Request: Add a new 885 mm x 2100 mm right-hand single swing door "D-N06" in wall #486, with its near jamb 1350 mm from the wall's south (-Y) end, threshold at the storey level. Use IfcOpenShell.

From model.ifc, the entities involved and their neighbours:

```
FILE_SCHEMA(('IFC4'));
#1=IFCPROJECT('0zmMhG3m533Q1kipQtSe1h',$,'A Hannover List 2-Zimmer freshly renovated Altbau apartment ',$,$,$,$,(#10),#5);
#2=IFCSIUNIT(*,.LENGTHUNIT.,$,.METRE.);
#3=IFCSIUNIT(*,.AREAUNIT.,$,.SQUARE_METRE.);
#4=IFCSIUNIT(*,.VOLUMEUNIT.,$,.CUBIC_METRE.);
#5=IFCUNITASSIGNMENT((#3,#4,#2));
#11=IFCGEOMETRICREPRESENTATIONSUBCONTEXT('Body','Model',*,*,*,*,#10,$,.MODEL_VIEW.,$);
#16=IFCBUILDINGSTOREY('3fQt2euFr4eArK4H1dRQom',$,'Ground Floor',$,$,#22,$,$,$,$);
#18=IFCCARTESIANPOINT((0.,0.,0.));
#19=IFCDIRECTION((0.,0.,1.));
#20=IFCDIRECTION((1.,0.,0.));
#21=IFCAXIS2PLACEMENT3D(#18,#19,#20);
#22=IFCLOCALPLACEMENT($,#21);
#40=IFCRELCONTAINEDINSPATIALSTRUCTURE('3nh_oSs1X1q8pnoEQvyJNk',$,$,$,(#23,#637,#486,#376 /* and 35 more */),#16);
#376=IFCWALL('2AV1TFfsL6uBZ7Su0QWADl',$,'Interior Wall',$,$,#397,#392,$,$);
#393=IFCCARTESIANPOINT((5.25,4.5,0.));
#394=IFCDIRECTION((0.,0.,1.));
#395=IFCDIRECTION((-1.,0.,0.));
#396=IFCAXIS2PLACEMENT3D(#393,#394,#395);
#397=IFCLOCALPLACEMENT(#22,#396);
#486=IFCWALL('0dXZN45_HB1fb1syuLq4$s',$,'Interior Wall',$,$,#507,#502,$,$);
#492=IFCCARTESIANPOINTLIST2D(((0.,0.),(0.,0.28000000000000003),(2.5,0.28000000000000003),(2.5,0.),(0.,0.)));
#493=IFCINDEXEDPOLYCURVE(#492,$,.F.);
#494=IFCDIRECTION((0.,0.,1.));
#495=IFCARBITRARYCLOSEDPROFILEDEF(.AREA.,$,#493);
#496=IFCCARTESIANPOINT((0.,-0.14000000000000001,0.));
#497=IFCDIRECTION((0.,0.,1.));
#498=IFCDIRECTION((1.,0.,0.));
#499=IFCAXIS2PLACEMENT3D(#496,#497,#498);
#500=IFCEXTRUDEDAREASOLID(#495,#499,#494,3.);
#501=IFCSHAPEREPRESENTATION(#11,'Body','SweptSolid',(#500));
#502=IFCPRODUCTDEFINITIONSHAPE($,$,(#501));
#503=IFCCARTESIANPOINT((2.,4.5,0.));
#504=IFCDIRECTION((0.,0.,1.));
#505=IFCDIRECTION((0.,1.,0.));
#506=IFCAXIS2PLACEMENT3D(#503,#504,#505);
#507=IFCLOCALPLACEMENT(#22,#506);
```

```python
import numpy as np
import ifcopenshell
import ifcopenshell.api.feature
import ifcopenshell.api.geometry
import ifcopenshell.api.root
import ifcopenshell.api.spatial
import ifcopenshell.geom
import ifcopenshell.util.element
import ifcopenshell.util.placement
import ifcopenshell.util.representation
import ifcopenshell.util.shape
import ifcopenshell.util.unit

model = ifcopenshell.open("model.ifc")
unit_scale = ifcopenshell.util.unit.calculate_unit_scale(model)
settings = ifcopenshell.geom.settings()


def volume(element):
    """Net volume in cubic metres, openings subtracted."""
    shape = ifcopenshell.geom.create_shape(settings, element)
    return ifcopenshell.util.shape.get_volume(shape.geometry)


wall = model.by_guid("0dXZN45_HB1fb1syuLq4$s")
storey = ifcopenshell.util.element.get_container(wall, ifc_class="IfcBuildingStorey")
context = ifcopenshell.util.representation.get_context(model, "Model", "Body", "MODEL_VIEW")
before = volume(wall)

width, height, from_end, sill = 0.885, 2.1, 1.35, 0.0  # metres

# The wall runs along its own X axis, and the end named is its -X end.
wall_shape = ifcopenshell.geom.create_shape(settings, wall)
x, y, z = ifcopenshell.util.shape.get_vertices(wall_shape.geometry).T
start = x.min() + from_end
face, thickness = float(y.min()), float(y.max() - y.min())
wall_matrix = ifcopenshell.util.placement.get_local_placement(wall.ObjectPlacement)
level = ifcopenshell.util.placement.get_local_placement(storey.ObjectPlacement)[2, 3]


def in_wall(x, y):
    """Placement at x, y metres in the wall's axes, at sill height."""
    matrix = wall_matrix.copy()
    matrix[:, 3] = wall_matrix @ np.array([x / unit_scale, y / unit_scale, 0.0, 1.0])
    matrix[2, 3] = level + sill / unit_scale
    return matrix


# Opening: a box that overshoots both wall faces by 50 mm.
opening = ifcopenshell.api.root.create_entity(model, ifc_class="IfcOpeningElement", predefined_type="OPENING")
box = ifcopenshell.api.geometry.add_wall_representation(
    model, context=context, length=width, height=height, thickness=thickness + 0.1
)
ifcopenshell.api.geometry.assign_representation(model, product=opening, representation=box)
ifcopenshell.api.geometry.edit_object_placement(model, product=opening, matrix=in_wall(start, face - 0.05), is_si=False)
ifcopenshell.api.feature.add_feature(model, feature=opening, element=wall)

door = ifcopenshell.api.root.create_entity(model, ifc_class="IfcDoor", name="D-N06", predefined_type="DOOR")
door.OverallWidth, door.OverallHeight = width / unit_scale, height / unit_scale
door.OperationType = "SINGLE_SWING_RIGHT"
body = ifcopenshell.api.geometry.add_door_representation(
    model,
    context=context,
    overall_width=door.OverallWidth,
    overall_height=door.OverallHeight,
    operation_type="SINGLE_SWING_RIGHT",
    lining_properties={"LiningDepth": thickness / unit_scale, "ThresholdDepth": thickness / unit_scale},
)
ifcopenshell.api.geometry.assign_representation(model, product=door, representation=body)
ifcopenshell.api.spatial.assign_container(model, products=[door], relating_structure=storey)
ifcopenshell.api.feature.add_filling(model, opening=opening, element=door)

# The lining spans the wall, so the door starts at the wall face.
ifcopenshell.api.geometry.edit_object_placement(model, product=door, matrix=in_wall(start, face), is_si=False)

after = volume(wall)

print(f"wall volume {before:.3f} -> {after:.3f} m3")

model.write("model_edited.ifc")
```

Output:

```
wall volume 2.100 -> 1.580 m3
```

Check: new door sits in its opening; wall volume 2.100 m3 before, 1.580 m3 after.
